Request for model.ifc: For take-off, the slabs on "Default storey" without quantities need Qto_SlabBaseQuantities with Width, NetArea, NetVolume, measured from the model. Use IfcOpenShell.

First a look at what the model holds.

```python
import ifcopenshell
import ifcopenshell.util.element
import ifcopenshell.util.unit

model = ifcopenshell.open("model.ifc")
print(model.schema)
for unit_type in ("LENGTHUNIT", "AREAUNIT", "VOLUMEUNIT"):
    print(unit_type, ifcopenshell.util.unit.calculate_unit_scale(model, unit_type))
storey = next(s for s in model.by_type("IfcBuildingStorey") if s.Name == "Default storey")
slabs = [e for e in ifcopenshell.util.element.get_decomposition(storey) if e.is_a("IfcSlab")]
for e in sorted(slabs, key=lambda e: e.id()):
    print(e.id(), e.is_a(), e.Name, list(ifcopenshell.util.element.get_psets(e, qtos_only=True)), sep=" | ")
```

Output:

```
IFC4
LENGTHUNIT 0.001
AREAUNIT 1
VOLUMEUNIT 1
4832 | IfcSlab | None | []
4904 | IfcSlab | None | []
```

```python
import ifcopenshell
import ifcopenshell.api.pset
import ifcopenshell.geom
import ifcopenshell.util.element
import ifcopenshell.util.shape
import ifcopenshell.util.unit

model = ifcopenshell.open("model.ifc")
unit_scale = ifcopenshell.util.unit.calculate_unit_scale(model)
area_scale = ifcopenshell.util.unit.calculate_unit_scale(model, "AREAUNIT")
volume_scale = ifcopenshell.util.unit.calculate_unit_scale(model, "VOLUMEUNIT")
settings = ifcopenshell.geom.settings()

storey = next(s for s in model.by_type("IfcBuildingStorey") if s.Name == "Default storey")
slabs = [e for e in ifcopenshell.util.element.get_decomposition(storey) if e.is_a("IfcSlab")]

for e in sorted(slabs, key=lambda e: e.id()):
    if ifcopenshell.util.element.get_psets(e, qtos_only=True, should_inherit=False):
        continue
    # Geometry comes back in metres, in the element's own axes.
    shape = ifcopenshell.geom.create_shape(settings, e)
    values = {
        "Width": ifcopenshell.util.shape.get_z(shape.geometry) / unit_scale,
        "NetArea": ifcopenshell.util.shape.get_footprint_area(shape.geometry) / area_scale,
        "NetVolume": ifcopenshell.util.shape.get_volume(shape.geometry) / volume_scale,
    }
    qto = ifcopenshell.api.pset.add_qto(model, product=e, name="Qto_SlabBaseQuantities")
    ifcopenshell.api.pset.edit_qto(model, qto=qto, properties=values)
    print(e.id(), {k: round(v, 3) for k, v in values.items()})

model.write("model_updated.ifc")
```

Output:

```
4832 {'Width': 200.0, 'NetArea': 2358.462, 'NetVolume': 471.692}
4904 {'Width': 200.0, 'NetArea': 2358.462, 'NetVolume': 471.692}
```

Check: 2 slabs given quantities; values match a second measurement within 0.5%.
